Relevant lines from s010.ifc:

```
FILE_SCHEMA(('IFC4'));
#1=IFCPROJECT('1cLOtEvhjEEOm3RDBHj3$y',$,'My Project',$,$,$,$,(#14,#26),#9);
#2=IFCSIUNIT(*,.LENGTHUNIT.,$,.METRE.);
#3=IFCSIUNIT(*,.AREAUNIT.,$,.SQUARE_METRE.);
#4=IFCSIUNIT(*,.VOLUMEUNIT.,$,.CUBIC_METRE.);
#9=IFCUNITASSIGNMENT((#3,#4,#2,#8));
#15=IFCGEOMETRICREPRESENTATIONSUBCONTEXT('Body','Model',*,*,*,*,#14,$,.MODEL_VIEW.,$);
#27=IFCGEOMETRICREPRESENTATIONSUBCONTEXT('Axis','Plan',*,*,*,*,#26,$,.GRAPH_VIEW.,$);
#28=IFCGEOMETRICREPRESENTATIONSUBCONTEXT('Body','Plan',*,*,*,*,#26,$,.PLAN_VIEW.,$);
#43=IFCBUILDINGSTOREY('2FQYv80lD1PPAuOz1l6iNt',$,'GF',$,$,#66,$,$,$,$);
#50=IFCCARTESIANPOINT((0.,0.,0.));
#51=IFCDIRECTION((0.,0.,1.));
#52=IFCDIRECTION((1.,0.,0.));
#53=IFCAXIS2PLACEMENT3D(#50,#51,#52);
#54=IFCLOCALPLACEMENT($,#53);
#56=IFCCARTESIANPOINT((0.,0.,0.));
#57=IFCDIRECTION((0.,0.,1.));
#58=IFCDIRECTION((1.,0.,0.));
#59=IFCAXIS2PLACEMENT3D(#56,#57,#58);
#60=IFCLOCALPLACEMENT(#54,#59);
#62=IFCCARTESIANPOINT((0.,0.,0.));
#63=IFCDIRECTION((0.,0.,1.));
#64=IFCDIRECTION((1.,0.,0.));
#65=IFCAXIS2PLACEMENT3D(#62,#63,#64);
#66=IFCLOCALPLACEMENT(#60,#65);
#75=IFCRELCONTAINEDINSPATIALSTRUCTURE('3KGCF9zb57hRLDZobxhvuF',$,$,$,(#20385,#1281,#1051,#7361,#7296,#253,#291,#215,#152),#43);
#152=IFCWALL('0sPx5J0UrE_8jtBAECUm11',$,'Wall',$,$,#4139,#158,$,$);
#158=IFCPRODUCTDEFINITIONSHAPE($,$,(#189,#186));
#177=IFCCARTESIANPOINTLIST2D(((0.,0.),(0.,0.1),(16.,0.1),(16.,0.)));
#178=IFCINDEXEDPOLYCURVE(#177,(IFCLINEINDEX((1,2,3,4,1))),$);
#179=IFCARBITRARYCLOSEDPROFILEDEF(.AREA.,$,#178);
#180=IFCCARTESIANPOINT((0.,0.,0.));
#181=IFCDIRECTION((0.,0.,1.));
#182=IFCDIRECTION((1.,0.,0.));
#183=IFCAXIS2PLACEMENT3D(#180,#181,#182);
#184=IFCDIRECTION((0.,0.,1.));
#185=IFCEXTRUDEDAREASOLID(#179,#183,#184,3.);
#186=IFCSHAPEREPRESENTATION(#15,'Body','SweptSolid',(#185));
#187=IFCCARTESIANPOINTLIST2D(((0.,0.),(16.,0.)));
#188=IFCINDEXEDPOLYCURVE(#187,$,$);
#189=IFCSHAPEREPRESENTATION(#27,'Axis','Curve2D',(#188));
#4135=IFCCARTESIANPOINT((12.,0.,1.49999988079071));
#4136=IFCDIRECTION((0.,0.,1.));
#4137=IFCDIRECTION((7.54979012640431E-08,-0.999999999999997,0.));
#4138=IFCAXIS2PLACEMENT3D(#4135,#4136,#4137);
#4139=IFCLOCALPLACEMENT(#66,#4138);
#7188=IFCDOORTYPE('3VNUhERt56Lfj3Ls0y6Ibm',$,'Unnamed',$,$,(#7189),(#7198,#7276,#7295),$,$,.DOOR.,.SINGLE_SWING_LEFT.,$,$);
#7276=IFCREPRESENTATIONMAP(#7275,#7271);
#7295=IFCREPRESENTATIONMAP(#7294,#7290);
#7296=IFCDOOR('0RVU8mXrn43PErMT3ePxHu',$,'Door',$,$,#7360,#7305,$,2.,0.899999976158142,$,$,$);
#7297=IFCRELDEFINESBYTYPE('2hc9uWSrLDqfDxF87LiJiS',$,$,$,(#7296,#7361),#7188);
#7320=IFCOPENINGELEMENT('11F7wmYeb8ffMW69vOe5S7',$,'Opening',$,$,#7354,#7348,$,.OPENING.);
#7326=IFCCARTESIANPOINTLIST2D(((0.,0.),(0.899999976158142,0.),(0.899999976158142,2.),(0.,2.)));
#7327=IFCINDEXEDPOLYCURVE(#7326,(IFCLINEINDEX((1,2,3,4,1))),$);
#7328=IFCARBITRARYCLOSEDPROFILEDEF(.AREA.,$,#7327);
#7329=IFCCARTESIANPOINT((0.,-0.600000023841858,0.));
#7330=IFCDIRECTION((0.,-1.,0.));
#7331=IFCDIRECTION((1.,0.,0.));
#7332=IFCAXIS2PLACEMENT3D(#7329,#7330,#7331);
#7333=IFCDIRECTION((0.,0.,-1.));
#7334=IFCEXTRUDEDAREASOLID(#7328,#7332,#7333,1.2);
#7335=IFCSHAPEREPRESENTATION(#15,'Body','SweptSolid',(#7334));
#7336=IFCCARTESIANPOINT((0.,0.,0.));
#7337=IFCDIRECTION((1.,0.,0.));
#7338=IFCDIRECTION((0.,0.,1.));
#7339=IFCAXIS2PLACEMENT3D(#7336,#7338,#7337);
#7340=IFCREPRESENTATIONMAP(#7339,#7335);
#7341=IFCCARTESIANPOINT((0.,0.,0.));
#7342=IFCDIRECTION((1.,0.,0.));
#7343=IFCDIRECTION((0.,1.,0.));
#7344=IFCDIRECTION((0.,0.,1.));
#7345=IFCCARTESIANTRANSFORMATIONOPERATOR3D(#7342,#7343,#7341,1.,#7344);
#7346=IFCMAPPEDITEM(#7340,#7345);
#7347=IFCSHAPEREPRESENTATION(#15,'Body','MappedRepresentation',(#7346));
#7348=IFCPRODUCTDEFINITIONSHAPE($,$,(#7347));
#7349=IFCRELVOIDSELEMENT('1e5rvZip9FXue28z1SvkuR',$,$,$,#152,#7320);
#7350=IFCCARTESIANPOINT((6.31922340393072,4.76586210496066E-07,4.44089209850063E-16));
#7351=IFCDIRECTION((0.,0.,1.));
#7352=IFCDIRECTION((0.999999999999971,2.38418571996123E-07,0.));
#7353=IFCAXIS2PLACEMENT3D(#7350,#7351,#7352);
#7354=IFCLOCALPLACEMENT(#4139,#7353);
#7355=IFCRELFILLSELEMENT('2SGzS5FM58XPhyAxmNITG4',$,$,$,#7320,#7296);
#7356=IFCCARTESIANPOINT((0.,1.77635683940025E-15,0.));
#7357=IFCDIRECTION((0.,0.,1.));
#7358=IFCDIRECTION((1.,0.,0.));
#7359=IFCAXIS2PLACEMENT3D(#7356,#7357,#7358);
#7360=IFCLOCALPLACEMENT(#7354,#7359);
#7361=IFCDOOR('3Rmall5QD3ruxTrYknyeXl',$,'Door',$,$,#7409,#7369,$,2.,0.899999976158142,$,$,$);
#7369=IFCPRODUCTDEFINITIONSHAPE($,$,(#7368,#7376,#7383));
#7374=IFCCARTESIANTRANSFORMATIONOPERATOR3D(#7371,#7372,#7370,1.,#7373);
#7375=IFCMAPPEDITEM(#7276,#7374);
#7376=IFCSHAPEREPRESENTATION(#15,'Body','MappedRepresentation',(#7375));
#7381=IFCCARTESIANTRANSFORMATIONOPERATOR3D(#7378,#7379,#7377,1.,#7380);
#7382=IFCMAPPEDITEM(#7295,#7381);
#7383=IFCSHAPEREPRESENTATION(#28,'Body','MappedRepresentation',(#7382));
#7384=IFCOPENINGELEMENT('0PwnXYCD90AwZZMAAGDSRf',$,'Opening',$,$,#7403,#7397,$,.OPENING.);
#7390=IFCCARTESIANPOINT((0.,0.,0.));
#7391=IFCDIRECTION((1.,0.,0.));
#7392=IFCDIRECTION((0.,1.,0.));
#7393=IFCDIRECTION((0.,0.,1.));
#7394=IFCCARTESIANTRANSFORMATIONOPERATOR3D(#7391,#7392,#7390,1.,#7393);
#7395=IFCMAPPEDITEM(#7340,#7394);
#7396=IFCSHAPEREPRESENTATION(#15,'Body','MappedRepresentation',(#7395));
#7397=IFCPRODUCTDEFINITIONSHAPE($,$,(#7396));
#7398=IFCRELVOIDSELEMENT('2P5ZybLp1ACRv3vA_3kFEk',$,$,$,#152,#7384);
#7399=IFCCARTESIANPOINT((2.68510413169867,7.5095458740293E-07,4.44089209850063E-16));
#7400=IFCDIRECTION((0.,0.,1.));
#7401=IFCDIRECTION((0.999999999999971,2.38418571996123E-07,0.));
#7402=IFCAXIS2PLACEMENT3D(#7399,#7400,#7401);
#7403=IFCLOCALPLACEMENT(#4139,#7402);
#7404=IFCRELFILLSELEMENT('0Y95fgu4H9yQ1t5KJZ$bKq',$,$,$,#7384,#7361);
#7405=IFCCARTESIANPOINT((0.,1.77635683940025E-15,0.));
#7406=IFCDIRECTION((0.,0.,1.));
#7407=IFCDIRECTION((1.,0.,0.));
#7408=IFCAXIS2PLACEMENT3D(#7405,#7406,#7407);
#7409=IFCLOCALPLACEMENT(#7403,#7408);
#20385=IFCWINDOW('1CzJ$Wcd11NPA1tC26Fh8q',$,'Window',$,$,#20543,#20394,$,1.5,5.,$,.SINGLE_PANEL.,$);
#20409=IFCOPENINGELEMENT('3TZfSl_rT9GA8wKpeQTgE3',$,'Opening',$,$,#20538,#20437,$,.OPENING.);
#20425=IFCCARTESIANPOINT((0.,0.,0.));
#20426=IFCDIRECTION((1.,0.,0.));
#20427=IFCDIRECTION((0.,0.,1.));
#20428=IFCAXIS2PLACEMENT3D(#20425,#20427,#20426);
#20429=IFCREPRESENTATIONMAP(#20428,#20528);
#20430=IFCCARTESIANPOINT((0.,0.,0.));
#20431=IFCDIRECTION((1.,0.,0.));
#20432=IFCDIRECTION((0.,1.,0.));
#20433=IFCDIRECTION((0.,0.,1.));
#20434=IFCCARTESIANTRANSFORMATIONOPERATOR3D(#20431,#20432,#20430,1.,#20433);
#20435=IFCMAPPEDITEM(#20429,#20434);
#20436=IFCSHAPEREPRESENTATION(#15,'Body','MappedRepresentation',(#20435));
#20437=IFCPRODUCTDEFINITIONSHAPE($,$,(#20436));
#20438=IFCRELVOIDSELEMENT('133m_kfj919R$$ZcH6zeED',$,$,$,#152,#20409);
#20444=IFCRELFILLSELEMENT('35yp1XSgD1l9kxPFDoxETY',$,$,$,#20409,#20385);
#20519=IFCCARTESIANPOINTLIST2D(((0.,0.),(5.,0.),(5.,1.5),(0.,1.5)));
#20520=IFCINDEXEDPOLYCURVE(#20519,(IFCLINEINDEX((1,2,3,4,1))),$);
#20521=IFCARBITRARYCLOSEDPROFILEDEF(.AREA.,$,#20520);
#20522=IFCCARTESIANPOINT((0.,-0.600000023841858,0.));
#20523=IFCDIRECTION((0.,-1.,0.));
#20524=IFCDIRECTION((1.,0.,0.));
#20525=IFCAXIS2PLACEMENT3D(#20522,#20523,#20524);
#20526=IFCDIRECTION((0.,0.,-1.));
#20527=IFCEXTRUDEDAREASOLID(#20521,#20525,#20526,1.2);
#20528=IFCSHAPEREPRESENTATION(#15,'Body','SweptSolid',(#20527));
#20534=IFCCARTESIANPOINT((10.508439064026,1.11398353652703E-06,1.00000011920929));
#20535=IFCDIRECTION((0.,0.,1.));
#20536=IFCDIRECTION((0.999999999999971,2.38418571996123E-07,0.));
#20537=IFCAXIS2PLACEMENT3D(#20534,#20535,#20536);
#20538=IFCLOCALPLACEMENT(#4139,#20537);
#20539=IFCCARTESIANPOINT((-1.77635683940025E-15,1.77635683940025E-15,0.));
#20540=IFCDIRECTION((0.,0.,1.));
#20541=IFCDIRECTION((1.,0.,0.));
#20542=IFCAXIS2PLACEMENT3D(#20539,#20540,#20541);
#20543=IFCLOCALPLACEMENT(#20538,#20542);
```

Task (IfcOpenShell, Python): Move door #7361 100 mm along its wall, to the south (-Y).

```python
import ifcopenshell
import ifcopenshell.api.geometry
import ifcopenshell.util.placement
import ifcopenshell.util.unit

model = ifcopenshell.open("s010.ifc")
unit_scale = ifcopenshell.util.unit.calculate_unit_scale(model)

door = model.by_guid("3Rmall5QD3ruxTrYknyeXl")
opening = door.FillsVoids[0].RelatingOpeningElement
wall = opening.VoidsElements[0].RelatingBuildingElement

wall_matrix = ifcopenshell.util.placement.get_local_placement(wall.ObjectPlacement)
shift = wall_matrix[:3, 0] * 0.1 / unit_scale
before = ifcopenshell.util.placement.get_local_placement(door.ObjectPlacement)[:3, 3].copy()

# The door is placed relative to its opening, so it follows when the opening moves.
matrix = ifcopenshell.util.placement.get_local_placement(opening.ObjectPlacement)
matrix[:3, 3] += shift
ifcopenshell.api.geometry.edit_object_placement(
    model, product=opening, matrix=matrix, is_si=False, should_transform_children=True
)

after = ifcopenshell.util.placement.get_local_placement(door.ObjectPlacement)[:3, 3]
print("door moved by", (after - before).round(3) + 0.0)

model.write("s010_edited.ifc")
```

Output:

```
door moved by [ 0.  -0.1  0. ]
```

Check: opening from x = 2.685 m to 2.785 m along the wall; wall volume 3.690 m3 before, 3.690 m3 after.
